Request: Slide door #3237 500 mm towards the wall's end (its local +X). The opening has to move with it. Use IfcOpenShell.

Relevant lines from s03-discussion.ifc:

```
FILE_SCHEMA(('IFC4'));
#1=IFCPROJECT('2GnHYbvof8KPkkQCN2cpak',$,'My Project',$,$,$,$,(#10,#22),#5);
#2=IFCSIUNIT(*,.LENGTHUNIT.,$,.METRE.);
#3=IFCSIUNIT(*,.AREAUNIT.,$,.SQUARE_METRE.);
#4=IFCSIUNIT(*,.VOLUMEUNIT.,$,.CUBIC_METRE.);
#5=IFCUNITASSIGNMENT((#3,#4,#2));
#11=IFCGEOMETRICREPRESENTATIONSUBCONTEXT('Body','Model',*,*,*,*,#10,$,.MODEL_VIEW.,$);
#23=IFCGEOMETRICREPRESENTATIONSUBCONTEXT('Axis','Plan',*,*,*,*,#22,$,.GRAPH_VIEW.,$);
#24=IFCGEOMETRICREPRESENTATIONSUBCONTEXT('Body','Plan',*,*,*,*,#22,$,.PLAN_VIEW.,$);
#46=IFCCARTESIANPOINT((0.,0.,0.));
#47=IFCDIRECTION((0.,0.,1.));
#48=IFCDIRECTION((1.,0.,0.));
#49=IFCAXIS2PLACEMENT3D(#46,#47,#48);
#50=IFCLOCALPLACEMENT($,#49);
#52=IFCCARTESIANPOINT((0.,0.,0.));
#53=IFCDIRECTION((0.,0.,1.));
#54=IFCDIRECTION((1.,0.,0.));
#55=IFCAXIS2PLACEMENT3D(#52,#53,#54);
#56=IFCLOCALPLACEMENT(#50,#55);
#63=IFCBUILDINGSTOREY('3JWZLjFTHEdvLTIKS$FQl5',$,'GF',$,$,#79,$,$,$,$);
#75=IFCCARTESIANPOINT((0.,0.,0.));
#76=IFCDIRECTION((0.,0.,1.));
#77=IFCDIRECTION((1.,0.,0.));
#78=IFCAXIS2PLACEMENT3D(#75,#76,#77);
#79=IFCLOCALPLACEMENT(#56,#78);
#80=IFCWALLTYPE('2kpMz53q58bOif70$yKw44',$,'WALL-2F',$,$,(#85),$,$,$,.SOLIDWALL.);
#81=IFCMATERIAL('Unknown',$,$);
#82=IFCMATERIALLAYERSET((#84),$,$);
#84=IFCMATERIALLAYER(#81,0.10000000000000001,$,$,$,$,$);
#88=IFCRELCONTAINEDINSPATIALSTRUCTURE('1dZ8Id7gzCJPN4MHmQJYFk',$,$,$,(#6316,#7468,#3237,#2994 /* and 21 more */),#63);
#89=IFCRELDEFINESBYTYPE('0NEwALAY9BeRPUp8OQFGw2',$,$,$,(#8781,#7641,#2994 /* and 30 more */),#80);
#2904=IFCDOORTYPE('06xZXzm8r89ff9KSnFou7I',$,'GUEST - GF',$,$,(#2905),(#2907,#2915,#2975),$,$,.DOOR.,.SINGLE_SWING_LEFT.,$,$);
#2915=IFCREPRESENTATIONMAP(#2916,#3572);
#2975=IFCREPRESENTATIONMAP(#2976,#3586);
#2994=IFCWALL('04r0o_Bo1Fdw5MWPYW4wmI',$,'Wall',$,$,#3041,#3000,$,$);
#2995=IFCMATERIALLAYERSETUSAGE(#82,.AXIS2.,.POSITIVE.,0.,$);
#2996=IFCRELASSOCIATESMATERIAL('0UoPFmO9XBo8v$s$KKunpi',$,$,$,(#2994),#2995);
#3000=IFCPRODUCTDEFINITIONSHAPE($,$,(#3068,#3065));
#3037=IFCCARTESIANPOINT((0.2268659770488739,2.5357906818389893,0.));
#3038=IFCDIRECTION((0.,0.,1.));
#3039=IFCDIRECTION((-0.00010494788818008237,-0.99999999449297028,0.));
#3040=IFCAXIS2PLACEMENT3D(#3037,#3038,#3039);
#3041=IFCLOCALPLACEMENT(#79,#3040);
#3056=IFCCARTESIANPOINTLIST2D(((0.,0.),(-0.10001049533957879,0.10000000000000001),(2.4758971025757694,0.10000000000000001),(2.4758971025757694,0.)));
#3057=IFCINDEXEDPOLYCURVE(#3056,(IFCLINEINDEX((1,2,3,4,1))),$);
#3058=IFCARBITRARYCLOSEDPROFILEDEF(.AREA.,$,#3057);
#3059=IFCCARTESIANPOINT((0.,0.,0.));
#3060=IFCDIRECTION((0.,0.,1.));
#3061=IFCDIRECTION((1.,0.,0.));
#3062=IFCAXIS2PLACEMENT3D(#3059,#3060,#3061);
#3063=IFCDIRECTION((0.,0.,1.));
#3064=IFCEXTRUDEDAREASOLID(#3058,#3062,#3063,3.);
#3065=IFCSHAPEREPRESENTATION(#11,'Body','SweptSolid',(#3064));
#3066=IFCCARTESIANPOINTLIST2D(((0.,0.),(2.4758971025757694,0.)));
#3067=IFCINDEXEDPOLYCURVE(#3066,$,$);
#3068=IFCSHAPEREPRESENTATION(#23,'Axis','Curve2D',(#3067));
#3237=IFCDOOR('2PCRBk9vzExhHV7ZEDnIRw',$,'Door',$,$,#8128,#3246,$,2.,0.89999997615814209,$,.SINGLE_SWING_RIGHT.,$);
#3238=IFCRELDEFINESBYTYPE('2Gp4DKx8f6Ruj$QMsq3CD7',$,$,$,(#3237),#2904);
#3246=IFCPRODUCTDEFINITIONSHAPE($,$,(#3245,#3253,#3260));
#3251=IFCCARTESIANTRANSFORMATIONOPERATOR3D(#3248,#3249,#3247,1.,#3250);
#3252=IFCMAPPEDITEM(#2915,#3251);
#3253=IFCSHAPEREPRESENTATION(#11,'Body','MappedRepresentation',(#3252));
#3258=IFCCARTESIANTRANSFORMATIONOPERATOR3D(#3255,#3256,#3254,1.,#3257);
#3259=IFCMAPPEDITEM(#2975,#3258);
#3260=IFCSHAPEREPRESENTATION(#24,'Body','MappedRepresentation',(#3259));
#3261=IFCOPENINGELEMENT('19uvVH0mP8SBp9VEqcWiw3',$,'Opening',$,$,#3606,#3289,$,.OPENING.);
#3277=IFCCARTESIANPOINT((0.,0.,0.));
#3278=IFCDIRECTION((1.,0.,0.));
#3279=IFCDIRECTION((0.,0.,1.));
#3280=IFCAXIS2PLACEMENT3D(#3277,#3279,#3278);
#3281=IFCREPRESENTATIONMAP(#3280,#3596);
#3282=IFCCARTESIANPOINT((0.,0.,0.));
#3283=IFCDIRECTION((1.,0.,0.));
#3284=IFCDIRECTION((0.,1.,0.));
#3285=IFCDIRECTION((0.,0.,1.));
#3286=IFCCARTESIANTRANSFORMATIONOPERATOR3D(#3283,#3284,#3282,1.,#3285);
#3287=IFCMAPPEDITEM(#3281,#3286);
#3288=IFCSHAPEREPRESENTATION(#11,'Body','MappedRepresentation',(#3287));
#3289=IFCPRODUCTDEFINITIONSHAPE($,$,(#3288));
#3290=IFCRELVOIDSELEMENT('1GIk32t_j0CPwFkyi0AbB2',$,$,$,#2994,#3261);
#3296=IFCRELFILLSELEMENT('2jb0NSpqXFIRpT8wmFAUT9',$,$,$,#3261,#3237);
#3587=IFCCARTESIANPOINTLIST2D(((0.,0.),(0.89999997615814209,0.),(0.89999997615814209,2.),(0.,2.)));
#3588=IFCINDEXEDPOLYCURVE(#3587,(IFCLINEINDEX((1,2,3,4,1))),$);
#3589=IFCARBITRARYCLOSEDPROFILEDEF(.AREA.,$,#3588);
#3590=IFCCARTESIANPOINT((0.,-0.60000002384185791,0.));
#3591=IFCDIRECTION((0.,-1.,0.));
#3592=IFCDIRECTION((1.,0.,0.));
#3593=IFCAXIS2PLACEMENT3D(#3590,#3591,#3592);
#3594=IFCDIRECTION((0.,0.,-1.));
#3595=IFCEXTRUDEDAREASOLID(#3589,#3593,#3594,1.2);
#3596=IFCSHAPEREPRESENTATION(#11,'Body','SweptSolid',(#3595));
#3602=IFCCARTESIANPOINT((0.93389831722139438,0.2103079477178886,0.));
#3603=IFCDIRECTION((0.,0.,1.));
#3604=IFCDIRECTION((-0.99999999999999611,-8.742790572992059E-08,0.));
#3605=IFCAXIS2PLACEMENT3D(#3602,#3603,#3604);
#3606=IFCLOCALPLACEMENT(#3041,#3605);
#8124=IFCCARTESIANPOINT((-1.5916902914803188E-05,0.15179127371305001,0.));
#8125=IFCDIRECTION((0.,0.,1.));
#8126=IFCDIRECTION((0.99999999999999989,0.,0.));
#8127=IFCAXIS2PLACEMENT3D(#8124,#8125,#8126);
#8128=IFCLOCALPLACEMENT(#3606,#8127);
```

```python
import ifcopenshell
import ifcopenshell.api.geometry
import ifcopenshell.util.placement
import ifcopenshell.util.unit

model = ifcopenshell.open("s03-discussion.ifc")
unit_scale = ifcopenshell.util.unit.calculate_unit_scale(model)

door = model.by_guid("2PCRBk9vzExhHV7ZEDnIRw")
opening = door.FillsVoids[0].RelatingOpeningElement
wall = opening.VoidsElements[0].RelatingBuildingElement

wall_matrix = ifcopenshell.util.placement.get_local_placement(wall.ObjectPlacement)
shift = wall_matrix[:3, 0] * 0.5 / unit_scale
before = ifcopenshell.util.placement.get_local_placement(door.ObjectPlacement)[:3, 3].copy()

# The door is placed relative to its opening, so it follows when the opening moves.
matrix = ifcopenshell.util.placement.get_local_placement(opening.ObjectPlacement)
matrix[:3, 3] += shift
ifcopenshell.api.geometry.edit_object_placement(
    model, product=opening, matrix=matrix, is_si=False, should_transform_children=True
)

after = ifcopenshell.util.placement.get_local_placement(door.ObjectPlacement)[:3, 3]
print("door moved by", (after - before).round(3) + 0.0)

model.write("s03-discussion_updated.ifc")
```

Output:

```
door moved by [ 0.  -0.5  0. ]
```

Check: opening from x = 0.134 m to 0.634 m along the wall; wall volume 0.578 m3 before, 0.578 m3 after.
